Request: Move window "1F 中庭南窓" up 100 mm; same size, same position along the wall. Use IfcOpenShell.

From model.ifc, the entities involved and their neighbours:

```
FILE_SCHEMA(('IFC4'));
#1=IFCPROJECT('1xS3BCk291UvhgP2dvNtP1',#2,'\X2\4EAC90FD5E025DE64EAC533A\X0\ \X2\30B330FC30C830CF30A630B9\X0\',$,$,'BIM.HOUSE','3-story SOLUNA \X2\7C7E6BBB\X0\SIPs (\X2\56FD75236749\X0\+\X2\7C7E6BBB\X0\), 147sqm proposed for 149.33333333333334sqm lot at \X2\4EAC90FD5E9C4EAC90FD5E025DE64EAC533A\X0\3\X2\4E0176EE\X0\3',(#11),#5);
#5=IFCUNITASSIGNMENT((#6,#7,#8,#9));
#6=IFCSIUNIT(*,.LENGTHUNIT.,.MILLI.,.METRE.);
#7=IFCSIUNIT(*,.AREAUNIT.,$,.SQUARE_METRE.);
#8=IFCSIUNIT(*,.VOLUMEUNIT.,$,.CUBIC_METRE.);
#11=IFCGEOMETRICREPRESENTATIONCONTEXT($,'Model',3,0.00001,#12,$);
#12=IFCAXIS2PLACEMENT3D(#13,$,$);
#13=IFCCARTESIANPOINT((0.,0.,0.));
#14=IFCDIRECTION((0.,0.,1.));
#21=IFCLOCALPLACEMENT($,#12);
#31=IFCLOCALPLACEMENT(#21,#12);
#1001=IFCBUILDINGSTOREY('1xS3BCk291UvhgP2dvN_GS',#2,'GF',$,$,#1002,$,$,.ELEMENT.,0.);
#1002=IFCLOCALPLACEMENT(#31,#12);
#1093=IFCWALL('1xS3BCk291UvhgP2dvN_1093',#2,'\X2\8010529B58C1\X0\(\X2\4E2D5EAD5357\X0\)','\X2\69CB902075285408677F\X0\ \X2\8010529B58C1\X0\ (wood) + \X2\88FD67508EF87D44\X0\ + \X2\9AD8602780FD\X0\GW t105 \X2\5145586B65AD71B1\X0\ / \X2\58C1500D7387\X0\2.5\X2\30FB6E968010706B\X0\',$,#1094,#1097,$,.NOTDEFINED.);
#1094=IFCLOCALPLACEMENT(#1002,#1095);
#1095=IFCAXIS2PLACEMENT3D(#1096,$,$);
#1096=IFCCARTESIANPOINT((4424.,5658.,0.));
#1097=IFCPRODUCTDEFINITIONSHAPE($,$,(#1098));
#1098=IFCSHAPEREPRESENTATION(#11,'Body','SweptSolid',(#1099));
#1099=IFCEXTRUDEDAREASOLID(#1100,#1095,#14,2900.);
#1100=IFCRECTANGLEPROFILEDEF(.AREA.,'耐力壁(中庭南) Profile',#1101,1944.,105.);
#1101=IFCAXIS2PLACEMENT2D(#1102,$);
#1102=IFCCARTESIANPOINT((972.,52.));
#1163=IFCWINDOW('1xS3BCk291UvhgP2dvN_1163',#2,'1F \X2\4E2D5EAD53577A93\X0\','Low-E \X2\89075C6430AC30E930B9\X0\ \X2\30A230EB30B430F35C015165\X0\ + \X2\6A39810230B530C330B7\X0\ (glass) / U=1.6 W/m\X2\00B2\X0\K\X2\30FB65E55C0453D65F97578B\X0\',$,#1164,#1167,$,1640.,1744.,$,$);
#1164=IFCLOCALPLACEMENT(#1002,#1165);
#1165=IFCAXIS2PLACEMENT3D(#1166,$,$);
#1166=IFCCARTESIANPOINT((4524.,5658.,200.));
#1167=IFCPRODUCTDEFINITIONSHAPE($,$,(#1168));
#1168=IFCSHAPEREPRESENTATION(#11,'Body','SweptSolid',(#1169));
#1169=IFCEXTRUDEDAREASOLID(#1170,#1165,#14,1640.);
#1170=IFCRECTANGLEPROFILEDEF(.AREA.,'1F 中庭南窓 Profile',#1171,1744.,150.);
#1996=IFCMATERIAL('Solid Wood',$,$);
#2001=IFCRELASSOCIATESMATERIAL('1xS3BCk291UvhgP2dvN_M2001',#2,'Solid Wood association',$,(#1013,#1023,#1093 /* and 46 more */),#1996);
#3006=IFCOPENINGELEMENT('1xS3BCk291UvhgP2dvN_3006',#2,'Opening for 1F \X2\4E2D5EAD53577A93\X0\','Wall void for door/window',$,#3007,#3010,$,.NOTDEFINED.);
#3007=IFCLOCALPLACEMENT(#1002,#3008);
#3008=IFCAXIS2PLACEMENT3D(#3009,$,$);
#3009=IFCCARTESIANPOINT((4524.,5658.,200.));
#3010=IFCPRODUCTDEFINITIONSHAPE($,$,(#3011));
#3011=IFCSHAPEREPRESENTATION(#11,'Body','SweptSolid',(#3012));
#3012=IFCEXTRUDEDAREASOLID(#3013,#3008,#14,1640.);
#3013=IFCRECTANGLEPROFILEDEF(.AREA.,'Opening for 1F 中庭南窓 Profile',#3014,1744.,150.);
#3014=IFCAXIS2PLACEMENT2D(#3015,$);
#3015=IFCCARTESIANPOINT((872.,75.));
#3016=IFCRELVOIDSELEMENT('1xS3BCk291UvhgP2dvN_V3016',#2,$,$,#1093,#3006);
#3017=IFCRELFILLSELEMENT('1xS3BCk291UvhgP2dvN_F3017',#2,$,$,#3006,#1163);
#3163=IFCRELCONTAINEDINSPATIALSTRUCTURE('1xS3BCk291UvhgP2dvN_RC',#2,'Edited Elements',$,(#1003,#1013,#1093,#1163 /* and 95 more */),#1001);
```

```python
import numpy as np
import ifcopenshell
import ifcopenshell.api.geometry
import ifcopenshell.util.placement
import ifcopenshell.util.unit

model = ifcopenshell.open("model.ifc")
unit_scale = ifcopenshell.util.unit.calculate_unit_scale(model)

window = model.by_guid("1xS3BCk291UvhgP2dvN_1163")
opening = window.FillsVoids[0].RelatingOpeningElement
dz = 100.0

shift = np.array([0.0, 0.0, dz])
# The window is not placed relative to its opening, so move both.
for product in (opening, window):
    matrix = ifcopenshell.util.placement.get_local_placement(product.ObjectPlacement)
    matrix[:3, 3] += shift
    ifcopenshell.api.geometry.edit_object_placement(model, product=product, matrix=matrix, is_si=False)

print(f"moved by {dz * unit_scale:+.3f} m")

model.write("model-out.ifc")
```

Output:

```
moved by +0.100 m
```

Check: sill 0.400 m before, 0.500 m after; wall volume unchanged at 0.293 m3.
